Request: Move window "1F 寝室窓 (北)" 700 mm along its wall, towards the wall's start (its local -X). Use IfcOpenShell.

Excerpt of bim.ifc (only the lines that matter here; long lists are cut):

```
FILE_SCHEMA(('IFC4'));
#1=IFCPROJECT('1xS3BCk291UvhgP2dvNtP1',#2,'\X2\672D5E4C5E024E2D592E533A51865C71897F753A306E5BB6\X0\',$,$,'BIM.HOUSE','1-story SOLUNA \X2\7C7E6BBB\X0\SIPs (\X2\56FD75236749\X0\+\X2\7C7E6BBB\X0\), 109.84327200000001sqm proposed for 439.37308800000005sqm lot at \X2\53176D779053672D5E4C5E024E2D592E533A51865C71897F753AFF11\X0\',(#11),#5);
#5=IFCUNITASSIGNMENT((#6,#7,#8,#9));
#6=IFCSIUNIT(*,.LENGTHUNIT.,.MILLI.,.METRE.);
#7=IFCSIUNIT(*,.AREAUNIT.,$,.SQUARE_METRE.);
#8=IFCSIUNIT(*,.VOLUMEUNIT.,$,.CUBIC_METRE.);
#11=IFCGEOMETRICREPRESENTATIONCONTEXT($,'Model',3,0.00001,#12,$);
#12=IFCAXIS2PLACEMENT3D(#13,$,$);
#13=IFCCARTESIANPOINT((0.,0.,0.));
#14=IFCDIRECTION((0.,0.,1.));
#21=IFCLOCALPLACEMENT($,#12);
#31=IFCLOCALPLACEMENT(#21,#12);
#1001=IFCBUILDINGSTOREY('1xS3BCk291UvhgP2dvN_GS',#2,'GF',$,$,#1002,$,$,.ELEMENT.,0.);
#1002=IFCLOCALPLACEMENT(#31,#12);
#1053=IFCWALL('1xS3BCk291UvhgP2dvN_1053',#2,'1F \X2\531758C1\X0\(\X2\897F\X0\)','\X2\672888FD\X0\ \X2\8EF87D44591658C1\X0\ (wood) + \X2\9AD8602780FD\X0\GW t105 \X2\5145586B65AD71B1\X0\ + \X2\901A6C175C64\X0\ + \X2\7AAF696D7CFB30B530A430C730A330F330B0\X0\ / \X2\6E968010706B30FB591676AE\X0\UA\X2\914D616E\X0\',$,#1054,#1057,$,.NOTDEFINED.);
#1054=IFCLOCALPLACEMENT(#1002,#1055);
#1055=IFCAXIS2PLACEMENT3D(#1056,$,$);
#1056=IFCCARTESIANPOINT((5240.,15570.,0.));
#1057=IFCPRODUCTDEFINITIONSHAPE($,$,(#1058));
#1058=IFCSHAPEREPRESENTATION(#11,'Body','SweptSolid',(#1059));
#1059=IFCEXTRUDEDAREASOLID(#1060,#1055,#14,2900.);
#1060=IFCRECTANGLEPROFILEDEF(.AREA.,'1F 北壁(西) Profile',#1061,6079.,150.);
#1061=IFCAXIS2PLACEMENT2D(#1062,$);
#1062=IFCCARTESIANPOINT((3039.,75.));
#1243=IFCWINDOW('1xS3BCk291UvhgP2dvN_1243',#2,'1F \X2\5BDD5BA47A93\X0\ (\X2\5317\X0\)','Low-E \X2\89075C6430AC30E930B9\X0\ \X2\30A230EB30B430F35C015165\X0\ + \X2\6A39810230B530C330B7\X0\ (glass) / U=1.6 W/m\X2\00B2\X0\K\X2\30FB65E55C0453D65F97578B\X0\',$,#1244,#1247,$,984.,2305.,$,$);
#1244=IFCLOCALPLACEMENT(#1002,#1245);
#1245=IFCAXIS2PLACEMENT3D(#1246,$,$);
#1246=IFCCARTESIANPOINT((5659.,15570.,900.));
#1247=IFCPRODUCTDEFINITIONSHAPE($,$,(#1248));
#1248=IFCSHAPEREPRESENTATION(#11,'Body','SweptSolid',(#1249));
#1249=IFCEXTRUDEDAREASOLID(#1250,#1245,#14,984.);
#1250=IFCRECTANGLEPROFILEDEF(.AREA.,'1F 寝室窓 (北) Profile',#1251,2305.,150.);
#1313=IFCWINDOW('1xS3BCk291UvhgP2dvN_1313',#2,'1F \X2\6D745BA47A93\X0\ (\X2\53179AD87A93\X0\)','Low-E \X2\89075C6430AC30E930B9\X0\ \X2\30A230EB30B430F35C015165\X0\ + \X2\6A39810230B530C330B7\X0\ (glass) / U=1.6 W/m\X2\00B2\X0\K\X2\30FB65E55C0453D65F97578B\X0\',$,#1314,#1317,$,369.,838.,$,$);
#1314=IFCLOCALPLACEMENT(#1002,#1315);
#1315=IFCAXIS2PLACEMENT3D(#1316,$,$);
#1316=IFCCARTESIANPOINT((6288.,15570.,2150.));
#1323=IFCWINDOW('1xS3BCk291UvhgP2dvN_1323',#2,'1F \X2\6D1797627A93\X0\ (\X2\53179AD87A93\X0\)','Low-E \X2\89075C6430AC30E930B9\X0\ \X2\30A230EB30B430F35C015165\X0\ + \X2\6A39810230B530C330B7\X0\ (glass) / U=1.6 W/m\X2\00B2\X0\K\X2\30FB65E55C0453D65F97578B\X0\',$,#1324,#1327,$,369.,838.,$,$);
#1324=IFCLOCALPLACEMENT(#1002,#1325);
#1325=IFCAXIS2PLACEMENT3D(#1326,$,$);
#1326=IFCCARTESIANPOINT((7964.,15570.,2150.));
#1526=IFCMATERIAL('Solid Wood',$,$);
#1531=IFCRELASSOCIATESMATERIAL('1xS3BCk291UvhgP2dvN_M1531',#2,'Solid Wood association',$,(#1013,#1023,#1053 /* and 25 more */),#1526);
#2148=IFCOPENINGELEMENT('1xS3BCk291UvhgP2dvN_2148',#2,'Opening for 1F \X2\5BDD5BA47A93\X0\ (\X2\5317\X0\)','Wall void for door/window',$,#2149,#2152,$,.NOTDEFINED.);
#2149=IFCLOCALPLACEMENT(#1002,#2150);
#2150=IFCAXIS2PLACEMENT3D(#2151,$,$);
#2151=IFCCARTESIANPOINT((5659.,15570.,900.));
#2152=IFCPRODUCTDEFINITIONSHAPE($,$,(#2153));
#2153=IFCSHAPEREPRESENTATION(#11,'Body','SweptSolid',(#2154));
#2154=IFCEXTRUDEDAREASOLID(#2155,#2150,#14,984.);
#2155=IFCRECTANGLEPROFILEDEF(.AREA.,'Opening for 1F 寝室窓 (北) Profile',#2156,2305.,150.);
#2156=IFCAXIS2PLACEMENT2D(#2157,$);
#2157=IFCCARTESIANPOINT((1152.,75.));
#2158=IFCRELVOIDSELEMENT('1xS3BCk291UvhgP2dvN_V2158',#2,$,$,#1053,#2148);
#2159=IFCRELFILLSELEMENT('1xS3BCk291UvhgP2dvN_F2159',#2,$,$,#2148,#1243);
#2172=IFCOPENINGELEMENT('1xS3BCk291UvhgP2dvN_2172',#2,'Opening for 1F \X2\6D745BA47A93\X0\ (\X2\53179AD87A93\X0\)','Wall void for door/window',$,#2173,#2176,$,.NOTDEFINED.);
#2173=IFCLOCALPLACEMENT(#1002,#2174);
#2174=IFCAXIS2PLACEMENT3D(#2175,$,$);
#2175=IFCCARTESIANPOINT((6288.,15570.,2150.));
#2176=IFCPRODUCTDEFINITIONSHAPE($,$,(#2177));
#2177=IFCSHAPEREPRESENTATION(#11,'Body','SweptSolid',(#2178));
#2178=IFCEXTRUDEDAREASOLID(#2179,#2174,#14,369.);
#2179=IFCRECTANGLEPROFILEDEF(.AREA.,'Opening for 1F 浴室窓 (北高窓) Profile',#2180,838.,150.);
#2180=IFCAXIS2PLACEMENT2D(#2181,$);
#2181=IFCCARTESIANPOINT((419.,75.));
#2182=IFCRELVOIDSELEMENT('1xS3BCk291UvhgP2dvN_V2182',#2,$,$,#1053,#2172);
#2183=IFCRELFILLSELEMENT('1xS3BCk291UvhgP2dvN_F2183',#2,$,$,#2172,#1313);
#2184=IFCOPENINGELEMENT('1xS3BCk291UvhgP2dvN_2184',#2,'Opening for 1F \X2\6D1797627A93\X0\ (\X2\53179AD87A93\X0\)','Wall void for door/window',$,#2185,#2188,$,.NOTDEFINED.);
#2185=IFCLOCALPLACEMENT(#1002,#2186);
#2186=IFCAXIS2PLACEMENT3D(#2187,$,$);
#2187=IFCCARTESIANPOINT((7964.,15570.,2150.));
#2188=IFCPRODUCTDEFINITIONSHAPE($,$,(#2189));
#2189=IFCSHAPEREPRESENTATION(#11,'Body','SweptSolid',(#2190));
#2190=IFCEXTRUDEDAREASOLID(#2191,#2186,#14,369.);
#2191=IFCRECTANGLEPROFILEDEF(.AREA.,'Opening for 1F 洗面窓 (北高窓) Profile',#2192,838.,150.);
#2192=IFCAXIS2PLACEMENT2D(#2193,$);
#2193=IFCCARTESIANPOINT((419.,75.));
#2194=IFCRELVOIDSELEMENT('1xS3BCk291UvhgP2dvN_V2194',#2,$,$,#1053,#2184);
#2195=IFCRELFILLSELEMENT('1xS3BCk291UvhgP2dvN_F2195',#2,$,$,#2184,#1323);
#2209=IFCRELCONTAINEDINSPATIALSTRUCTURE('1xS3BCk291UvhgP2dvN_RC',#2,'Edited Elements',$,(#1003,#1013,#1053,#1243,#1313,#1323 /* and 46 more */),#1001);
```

```python
import ifcopenshell
import ifcopenshell.api.geometry
import ifcopenshell.util.placement
import ifcopenshell.util.unit

model = ifcopenshell.open("bim.ifc")
unit_scale = ifcopenshell.util.unit.calculate_unit_scale(model)

window = model.by_guid("1xS3BCk291UvhgP2dvN_1243")
opening = window.FillsVoids[0].RelatingOpeningElement
wall = opening.VoidsElements[0].RelatingBuildingElement

wall_matrix = ifcopenshell.util.placement.get_local_placement(wall.ObjectPlacement)
shift = wall_matrix[:3, 0] * -0.7 / unit_scale
before = ifcopenshell.util.placement.get_local_placement(window.ObjectPlacement)[:3, 3].copy()

# The window is not placed relative to its opening, so move both.
for product in (opening, window):
    matrix = ifcopenshell.util.placement.get_local_placement(product.ObjectPlacement)
    matrix[:3, 3] += shift
    ifcopenshell.api.geometry.edit_object_placement(model, product=product, matrix=matrix, is_si=False)

after = ifcopenshell.util.placement.get_local_placement(window.ObjectPlacement)[:3, 3]
print("window moved by", (after - before).round(3) + 0.0)

model.write("bim-out.ifc")
```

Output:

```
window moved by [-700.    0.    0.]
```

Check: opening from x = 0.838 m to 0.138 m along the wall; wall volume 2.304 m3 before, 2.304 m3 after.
